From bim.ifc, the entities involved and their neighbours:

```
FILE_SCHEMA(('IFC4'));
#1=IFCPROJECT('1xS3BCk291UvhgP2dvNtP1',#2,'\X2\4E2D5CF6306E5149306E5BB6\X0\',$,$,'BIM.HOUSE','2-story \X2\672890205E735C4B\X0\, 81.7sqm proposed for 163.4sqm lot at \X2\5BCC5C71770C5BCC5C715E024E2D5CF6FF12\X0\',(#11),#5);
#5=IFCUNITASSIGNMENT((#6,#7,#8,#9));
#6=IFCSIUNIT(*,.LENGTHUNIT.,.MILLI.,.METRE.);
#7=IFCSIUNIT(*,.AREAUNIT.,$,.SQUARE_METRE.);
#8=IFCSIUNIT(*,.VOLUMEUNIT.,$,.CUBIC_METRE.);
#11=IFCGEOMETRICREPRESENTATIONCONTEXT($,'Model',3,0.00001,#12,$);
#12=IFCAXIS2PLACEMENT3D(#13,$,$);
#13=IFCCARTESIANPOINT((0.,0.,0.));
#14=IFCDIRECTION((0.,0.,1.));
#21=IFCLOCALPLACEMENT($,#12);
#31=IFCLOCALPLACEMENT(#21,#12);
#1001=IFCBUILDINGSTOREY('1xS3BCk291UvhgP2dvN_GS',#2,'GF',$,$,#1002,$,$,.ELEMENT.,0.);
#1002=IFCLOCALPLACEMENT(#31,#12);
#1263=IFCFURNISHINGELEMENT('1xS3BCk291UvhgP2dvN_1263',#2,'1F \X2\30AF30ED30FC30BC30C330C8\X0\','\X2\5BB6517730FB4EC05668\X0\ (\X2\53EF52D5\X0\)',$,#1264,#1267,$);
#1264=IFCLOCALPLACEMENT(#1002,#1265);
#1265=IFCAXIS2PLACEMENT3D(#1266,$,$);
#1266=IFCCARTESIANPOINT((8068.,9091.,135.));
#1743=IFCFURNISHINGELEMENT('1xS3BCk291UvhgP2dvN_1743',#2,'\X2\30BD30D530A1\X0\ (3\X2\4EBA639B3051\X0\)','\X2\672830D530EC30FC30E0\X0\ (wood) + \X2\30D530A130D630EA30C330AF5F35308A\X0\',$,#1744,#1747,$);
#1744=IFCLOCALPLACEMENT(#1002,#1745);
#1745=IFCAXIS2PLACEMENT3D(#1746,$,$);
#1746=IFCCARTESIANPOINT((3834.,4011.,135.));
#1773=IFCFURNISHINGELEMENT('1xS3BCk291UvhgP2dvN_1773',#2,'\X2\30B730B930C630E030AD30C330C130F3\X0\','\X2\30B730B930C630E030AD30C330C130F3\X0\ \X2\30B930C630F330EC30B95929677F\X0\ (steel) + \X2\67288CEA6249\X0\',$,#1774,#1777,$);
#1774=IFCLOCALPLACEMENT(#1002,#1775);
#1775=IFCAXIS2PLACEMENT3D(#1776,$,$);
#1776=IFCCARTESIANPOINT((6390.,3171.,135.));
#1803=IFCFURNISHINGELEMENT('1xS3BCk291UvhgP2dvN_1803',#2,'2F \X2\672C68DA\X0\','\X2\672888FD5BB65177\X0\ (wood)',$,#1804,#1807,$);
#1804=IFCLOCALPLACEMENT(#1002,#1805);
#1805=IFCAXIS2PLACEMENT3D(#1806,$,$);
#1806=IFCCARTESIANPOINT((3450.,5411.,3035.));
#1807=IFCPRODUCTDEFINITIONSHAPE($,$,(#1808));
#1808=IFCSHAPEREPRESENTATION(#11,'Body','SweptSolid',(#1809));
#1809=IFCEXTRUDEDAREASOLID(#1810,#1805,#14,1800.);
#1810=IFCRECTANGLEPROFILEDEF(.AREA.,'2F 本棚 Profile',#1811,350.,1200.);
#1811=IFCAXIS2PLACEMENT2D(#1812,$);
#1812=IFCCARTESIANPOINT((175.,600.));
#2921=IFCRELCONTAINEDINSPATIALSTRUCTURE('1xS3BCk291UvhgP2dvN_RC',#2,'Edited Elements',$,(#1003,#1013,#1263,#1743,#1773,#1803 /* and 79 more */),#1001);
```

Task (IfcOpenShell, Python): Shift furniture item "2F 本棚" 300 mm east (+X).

```python
import ifcopenshell
import ifcopenshell.api.geometry
import ifcopenshell.util.placement
import ifcopenshell.util.unit

model = ifcopenshell.open("bim.ifc")
unit_scale = ifcopenshell.util.unit.calculate_unit_scale(model)

item = model.by_id(1803)
matrix = ifcopenshell.util.placement.get_local_placement(item.ObjectPlacement)
matrix[0, 3] += 0.3 / unit_scale
ifcopenshell.api.geometry.edit_object_placement(model, product=item, matrix=matrix, is_si=False)

print(ifcopenshell.util.placement.get_local_placement(item.ObjectPlacement).round(3) + 0.0)

model.write("bim_updated.ifc")
```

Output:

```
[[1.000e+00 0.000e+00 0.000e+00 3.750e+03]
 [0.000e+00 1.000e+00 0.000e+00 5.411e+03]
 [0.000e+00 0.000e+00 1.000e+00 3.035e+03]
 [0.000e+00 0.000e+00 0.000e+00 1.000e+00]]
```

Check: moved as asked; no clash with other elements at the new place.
